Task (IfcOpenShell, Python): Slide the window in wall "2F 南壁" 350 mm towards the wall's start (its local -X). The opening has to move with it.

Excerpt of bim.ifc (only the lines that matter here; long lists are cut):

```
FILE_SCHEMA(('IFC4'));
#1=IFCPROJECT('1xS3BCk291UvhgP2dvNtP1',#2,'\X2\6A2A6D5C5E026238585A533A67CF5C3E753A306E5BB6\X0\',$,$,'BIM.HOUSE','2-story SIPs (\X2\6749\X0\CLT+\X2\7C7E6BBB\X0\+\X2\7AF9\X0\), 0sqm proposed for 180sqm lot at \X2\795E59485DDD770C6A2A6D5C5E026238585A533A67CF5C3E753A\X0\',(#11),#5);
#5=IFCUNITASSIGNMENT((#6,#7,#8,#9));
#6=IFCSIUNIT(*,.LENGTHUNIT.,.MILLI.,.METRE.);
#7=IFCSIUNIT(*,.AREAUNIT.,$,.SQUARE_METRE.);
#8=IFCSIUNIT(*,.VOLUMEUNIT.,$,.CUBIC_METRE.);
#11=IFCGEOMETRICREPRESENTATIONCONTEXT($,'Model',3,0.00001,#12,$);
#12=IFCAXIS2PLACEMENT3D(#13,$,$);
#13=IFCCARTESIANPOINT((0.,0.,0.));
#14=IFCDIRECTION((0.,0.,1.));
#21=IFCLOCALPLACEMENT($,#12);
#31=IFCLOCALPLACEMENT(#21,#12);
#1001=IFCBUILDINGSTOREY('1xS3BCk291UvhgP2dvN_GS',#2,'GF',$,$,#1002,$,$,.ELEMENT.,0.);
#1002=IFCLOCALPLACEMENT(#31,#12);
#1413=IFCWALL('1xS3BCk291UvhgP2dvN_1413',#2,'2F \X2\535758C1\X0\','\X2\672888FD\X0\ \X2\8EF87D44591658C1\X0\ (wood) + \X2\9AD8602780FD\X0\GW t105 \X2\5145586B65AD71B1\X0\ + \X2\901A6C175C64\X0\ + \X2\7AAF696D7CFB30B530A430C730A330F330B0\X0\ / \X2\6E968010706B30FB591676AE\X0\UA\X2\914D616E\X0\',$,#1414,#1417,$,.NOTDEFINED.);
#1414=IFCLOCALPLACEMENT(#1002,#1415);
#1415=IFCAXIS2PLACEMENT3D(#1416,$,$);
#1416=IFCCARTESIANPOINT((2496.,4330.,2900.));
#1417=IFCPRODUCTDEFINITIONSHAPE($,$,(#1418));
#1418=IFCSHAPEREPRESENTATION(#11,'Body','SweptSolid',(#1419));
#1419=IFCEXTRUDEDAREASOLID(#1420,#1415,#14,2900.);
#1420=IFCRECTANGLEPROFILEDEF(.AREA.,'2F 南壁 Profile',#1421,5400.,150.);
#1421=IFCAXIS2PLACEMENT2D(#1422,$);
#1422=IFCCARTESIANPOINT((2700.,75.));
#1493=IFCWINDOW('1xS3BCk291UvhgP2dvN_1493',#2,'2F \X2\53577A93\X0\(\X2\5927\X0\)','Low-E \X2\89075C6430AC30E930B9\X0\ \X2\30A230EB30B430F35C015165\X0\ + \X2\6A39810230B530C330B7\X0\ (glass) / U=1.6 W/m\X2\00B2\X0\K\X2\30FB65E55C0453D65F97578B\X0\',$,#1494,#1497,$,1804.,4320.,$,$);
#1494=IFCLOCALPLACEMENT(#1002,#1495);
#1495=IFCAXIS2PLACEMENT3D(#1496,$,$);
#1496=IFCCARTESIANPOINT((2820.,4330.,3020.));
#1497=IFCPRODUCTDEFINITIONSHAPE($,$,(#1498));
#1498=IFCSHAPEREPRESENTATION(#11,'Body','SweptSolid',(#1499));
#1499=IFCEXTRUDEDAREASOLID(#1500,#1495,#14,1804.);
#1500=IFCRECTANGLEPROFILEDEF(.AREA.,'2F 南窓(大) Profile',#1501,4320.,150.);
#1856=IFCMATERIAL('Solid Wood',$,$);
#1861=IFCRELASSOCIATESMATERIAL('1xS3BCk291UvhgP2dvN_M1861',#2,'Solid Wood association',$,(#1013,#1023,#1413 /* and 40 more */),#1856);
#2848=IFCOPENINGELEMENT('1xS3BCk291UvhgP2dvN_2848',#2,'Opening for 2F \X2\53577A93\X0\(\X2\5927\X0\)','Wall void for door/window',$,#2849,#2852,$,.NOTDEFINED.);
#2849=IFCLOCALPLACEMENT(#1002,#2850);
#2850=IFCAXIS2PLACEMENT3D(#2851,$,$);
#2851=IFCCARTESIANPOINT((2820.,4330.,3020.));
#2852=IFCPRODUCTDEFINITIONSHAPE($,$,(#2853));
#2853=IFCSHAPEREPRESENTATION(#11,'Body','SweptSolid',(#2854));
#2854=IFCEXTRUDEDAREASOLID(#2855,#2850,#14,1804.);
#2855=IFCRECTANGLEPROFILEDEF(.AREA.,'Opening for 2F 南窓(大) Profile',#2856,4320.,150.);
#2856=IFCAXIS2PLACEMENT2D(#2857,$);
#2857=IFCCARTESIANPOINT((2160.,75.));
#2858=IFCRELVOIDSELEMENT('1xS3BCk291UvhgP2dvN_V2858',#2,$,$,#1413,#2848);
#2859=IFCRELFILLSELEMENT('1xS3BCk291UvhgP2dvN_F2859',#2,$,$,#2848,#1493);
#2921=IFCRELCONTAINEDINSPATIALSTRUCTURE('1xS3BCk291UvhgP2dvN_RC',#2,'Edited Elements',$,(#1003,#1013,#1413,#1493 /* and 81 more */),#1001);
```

```python
import ifcopenshell
import ifcopenshell.api.geometry
import ifcopenshell.util.placement

model = ifcopenshell.open("bim.ifc")

window = model.by_id(1493)
opening = window.FillsVoids[0].RelatingOpeningElement
wall = opening.VoidsElements[0].RelatingBuildingElement

wall_matrix = ifcopenshell.util.placement.get_local_placement(wall.ObjectPlacement)
shift = wall_matrix[:3, 0] * -350.0
before = ifcopenshell.util.placement.get_local_placement(window.ObjectPlacement)[:3, 3].copy()

# The window is not placed relative to its opening, so move both.
for product in (opening, window):
    matrix = ifcopenshell.util.placement.get_local_placement(product.ObjectPlacement)
    matrix[:3, 3] += shift
    ifcopenshell.api.geometry.edit_object_placement(model, product=product, matrix=matrix, is_si=False)

after = ifcopenshell.util.placement.get_local_placement(window.ObjectPlacement)[:3, 3]
print("window moved by", (after - before).round(3) + 0.0)

model.write("bim_edited.ifc")
```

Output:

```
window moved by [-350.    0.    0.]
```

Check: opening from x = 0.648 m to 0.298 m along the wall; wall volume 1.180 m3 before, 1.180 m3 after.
